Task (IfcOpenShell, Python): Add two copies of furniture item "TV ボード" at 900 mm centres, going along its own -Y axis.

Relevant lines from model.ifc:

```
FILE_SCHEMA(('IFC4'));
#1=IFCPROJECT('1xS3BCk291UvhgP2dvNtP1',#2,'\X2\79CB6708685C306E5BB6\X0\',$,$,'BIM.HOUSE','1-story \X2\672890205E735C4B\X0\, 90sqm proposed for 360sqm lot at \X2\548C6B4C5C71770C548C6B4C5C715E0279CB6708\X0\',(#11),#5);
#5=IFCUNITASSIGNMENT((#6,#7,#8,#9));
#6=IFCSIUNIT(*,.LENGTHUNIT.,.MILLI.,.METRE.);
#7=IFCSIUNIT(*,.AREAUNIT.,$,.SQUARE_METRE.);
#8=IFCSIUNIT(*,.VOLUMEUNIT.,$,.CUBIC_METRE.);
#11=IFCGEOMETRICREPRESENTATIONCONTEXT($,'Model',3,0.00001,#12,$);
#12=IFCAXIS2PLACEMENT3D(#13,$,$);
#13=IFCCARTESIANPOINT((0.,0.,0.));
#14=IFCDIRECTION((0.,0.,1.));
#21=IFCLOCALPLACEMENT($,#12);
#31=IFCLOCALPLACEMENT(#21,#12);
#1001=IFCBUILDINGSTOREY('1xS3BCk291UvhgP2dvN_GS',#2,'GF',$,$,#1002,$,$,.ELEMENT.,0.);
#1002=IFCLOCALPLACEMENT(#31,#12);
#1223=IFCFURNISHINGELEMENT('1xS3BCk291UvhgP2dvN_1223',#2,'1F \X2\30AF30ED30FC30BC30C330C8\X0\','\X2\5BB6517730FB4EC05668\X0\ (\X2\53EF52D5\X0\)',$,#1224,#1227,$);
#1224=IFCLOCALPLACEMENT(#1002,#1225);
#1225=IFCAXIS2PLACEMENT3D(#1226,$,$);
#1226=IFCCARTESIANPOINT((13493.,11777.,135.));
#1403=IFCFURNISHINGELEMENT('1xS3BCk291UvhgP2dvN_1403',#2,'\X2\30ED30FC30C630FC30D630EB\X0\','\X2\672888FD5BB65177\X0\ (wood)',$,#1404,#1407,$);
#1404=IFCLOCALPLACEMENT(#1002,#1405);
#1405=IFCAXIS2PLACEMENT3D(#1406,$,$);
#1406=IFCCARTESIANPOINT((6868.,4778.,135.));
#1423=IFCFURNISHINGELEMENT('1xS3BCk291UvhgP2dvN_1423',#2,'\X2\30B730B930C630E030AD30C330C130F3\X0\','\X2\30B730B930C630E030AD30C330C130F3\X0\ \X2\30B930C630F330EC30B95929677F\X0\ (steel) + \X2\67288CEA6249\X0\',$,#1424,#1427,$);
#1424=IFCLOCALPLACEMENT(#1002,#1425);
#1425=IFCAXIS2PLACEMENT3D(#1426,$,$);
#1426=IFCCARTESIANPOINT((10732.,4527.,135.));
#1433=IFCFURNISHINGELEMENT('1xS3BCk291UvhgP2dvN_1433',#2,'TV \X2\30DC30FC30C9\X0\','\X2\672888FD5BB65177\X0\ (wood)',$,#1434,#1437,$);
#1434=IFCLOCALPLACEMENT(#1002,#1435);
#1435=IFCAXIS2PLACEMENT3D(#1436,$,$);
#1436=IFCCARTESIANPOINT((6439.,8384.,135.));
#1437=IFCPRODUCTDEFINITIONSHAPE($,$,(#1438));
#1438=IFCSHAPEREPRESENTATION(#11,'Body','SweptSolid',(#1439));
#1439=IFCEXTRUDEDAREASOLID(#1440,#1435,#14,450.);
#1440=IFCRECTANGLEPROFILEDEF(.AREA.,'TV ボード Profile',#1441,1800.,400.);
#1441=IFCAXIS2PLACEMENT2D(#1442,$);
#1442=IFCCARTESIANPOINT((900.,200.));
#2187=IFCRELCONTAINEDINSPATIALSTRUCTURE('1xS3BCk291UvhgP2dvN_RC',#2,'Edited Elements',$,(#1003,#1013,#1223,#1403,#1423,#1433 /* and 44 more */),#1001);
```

```python
import ifcopenshell
import ifcopenshell.api.geometry
import ifcopenshell.api.root
import ifcopenshell.util.element
import ifcopenshell.util.placement
import ifcopenshell.util.unit

model = ifcopenshell.open("model.ifc")
unit_scale = ifcopenshell.util.unit.calculate_unit_scale(model)


def reuse_history(source, copy):
    """copy_class also copies each property set's owner history, people and application; keep the originals."""
    for rel in copy.IsDefinedBy:
        if rel.is_a("IfcRelDefinesByProperties") and (history := rel.RelatingPropertyDefinition.OwnerHistory):
            rel.RelatingPropertyDefinition.OwnerHistory = source.OwnerHistory
            ifcopenshell.util.element.remove_deep2(model, history)


source = model.by_guid("1xS3BCk291UvhgP2dvN_1433")
base = ifcopenshell.util.placement.get_local_placement(source.ObjectPlacement)
step = -base[:3, 1] * 0.9 / unit_scale

for i in range(1, 3):
    copy = ifcopenshell.api.root.copy_class(model, product=source)
    copy.Representation = ifcopenshell.util.element.copy_deep(
        model, source.Representation, exclude=["IfcGeometricRepresentationContext", "IfcRepresentationMap"]
    )
    reuse_history(source, copy)
    matrix = base.copy()
    matrix[:3, 3] += i * step
    print("added at", matrix[:3, 3].round(3) + 0.0)
    ifcopenshell.api.geometry.edit_object_placement(model, product=copy, matrix=matrix, is_si=False)

model.write("model-out.ifc")
```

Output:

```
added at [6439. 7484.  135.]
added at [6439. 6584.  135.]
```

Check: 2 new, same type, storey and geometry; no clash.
